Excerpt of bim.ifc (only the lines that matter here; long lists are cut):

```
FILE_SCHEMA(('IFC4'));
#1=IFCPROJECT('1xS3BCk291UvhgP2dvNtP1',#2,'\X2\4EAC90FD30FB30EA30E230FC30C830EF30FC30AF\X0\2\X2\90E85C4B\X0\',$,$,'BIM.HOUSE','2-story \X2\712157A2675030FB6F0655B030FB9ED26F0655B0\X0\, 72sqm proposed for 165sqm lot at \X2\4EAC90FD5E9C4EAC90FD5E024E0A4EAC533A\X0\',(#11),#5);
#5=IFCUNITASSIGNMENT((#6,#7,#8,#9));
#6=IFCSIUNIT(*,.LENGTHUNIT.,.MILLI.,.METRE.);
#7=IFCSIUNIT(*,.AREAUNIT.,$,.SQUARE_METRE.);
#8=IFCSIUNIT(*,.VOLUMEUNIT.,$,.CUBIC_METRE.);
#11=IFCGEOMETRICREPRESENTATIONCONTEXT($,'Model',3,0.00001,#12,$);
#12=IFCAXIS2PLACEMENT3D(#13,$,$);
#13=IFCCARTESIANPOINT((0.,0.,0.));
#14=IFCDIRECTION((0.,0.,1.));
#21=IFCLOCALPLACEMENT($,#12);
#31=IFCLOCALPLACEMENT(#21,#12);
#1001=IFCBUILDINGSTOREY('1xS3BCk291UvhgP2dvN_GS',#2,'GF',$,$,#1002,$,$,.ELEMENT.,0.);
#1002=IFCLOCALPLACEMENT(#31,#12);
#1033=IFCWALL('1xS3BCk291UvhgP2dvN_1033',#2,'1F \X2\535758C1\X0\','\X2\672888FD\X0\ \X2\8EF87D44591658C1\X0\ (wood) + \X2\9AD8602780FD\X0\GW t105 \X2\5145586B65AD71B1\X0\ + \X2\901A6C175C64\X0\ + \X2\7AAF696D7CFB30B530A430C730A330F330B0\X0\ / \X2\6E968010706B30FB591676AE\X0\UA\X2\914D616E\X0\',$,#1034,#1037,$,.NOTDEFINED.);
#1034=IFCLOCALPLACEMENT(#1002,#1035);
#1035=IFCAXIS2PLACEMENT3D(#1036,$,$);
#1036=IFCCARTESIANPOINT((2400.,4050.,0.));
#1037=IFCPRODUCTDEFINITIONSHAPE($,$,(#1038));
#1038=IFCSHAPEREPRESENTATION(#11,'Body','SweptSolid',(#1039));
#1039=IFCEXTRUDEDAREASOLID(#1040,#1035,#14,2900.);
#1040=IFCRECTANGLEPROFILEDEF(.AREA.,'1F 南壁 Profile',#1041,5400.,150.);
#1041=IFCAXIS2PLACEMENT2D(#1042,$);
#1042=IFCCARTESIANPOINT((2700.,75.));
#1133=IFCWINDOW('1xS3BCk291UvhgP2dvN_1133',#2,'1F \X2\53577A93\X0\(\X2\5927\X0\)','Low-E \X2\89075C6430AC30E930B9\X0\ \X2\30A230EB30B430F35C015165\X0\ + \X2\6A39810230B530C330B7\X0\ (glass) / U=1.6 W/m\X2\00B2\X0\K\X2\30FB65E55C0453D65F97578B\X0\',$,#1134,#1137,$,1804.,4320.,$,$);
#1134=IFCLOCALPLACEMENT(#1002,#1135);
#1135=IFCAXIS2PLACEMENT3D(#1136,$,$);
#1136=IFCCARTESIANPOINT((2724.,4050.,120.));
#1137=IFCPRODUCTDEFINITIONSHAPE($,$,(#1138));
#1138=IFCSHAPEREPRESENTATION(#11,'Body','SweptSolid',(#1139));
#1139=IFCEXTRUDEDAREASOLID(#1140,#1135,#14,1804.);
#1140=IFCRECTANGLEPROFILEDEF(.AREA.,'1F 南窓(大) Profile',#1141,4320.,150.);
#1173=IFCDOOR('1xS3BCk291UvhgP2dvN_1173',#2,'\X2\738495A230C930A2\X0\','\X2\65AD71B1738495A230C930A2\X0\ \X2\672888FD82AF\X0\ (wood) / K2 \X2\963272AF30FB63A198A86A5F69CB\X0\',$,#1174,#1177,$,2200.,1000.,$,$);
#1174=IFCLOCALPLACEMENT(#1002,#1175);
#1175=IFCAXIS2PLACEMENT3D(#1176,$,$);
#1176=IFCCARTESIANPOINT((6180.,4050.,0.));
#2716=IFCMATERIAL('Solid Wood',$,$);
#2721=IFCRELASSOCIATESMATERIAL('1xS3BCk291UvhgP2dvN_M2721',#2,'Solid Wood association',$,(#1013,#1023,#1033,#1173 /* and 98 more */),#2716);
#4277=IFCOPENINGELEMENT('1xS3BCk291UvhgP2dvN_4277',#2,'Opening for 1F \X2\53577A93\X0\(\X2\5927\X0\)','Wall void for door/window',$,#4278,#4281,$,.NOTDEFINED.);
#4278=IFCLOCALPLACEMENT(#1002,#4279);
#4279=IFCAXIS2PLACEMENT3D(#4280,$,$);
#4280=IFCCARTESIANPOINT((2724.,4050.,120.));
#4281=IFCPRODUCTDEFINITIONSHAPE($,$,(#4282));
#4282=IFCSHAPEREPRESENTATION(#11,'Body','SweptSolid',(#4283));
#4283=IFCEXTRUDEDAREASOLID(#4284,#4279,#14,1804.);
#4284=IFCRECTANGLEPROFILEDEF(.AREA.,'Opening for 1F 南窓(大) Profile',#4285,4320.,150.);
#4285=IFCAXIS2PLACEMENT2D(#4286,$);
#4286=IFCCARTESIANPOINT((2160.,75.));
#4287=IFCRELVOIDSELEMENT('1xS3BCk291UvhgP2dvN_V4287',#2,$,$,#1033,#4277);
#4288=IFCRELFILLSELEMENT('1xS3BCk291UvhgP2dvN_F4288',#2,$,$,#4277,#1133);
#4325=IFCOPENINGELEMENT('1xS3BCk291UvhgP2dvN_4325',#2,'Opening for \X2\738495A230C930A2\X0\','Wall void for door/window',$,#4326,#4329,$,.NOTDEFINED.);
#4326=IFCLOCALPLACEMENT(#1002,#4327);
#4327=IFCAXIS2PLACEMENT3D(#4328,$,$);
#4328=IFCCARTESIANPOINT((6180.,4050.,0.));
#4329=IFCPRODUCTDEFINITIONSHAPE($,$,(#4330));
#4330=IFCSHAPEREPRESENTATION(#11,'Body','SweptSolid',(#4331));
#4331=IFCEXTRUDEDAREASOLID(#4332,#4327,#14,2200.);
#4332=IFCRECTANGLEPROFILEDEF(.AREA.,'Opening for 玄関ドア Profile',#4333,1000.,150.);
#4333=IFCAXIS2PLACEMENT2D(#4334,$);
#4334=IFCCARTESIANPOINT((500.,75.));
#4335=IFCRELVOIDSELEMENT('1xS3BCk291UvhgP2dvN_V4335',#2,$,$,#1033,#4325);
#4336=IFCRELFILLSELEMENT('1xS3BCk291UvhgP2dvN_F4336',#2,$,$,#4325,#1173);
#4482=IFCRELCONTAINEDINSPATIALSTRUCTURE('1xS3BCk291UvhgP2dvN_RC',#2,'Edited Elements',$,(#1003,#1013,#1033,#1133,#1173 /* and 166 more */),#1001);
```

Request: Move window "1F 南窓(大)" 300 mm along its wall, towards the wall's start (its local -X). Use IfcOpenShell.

```python
import ifcopenshell
import ifcopenshell.api.geometry
import ifcopenshell.util.placement

model = ifcopenshell.open("bim.ifc")

window = model.by_id(1133)
opening = window.FillsVoids[0].RelatingOpeningElement
wall = opening.VoidsElements[0].RelatingBuildingElement

wall_matrix = ifcopenshell.util.placement.get_local_placement(wall.ObjectPlacement)
shift = wall_matrix[:3, 0] * -300.0
before = ifcopenshell.util.placement.get_local_placement(window.ObjectPlacement)[:3, 3].copy()

# The window is not placed relative to its opening, so move both.
for product in (opening, window):
    matrix = ifcopenshell.util.placement.get_local_placement(product.ObjectPlacement)
    matrix[:3, 3] += shift
    ifcopenshell.api.geometry.edit_object_placement(model, product=product, matrix=matrix, is_si=False)

after = ifcopenshell.util.placement.get_local_placement(window.ObjectPlacement)[:3, 3]
print("window moved by", (after - before).round(3) + 0.0)

model.write("bim_v2.ifc")
```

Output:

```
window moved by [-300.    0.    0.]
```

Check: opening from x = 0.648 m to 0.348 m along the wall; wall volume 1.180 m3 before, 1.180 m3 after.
